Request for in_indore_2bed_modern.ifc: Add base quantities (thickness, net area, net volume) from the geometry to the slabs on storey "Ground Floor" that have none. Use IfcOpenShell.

First a look at what the model holds.

```python
import ifcopenshell
import ifcopenshell.util.element
import ifcopenshell.util.unit

model = ifcopenshell.open("in_indore_2bed_modern.ifc")
print(model.schema)
for unit_type in ("LENGTHUNIT", "AREAUNIT", "VOLUMEUNIT"):
    print(unit_type, ifcopenshell.util.unit.calculate_unit_scale(model, unit_type))
storey = next(s for s in model.by_type("IfcBuildingStorey") if s.Name == "Ground Floor")
slabs = [e for e in ifcopenshell.util.element.get_decomposition(storey) if e.is_a("IfcSlab")]
for e in sorted(slabs, key=lambda e: e.id()):
    print(e.id(), e.is_a(), e.Name, list(ifcopenshell.util.element.get_psets(e, qtos_only=True)), sep=" | ")
```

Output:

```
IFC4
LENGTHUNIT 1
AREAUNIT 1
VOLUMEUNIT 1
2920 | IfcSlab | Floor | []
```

```python
import ifcopenshell
import ifcopenshell.api.pset
import ifcopenshell.geom
import ifcopenshell.util.element
import ifcopenshell.util.shape
import ifcopenshell.util.unit

model = ifcopenshell.open("in_indore_2bed_modern.ifc")
unit_scale = ifcopenshell.util.unit.calculate_unit_scale(model)
area_scale = ifcopenshell.util.unit.calculate_unit_scale(model, "AREAUNIT")
volume_scale = ifcopenshell.util.unit.calculate_unit_scale(model, "VOLUMEUNIT")
settings = ifcopenshell.geom.settings()

storey = next(s for s in model.by_type("IfcBuildingStorey") if s.Name == "Ground Floor")
slabs = [e for e in ifcopenshell.util.element.get_decomposition(storey) if e.is_a("IfcSlab")]

for e in sorted(slabs, key=lambda e: e.id()):
    if ifcopenshell.util.element.get_psets(e, qtos_only=True, should_inherit=False):
        continue
    # Geometry comes back in metres, in the element's own axes.
    shape = ifcopenshell.geom.create_shape(settings, e)
    values = {
        "Width": ifcopenshell.util.shape.get_z(shape.geometry) / unit_scale,
        "NetArea": ifcopenshell.util.shape.get_footprint_area(shape.geometry) / area_scale,
        "NetVolume": ifcopenshell.util.shape.get_volume(shape.geometry) / volume_scale,
    }
    qto = ifcopenshell.api.pset.add_qto(model, product=e, name="Qto_SlabBaseQuantities")
    ifcopenshell.api.pset.edit_qto(model, qto=qto, properties=values)
    print(e.id(), {k: round(v, 3) for k, v in values.items()})

model.write("in_indore_2bed_modern-out.ifc")
```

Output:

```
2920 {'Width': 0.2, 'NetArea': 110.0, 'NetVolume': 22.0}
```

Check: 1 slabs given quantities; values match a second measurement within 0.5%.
